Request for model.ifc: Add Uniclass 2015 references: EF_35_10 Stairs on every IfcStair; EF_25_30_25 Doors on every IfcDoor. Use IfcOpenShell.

First a look at what the model holds.

```python
import ifcopenshell

model = ifcopenshell.open("model.ifc")
print(model.schema)
print("classifications:", [c.Name for c in model.by_type("IfcClassification")])
for ifc_class in ("IfcDoor", "IfcRoof", "IfcStair", "IfcWall", "IfcWindow"):
    print(ifc_class, len(model.by_type(ifc_class)))
```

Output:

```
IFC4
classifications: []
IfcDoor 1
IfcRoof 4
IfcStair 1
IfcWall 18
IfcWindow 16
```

```python
import ifcopenshell
import ifcopenshell.api.classification

model = ifcopenshell.open("model.ifc")

system = ifcopenshell.api.classification.add_classification(model, classification="Uniclass 2015")

codes = {
    "IfcStair": ("EF_35_10", "Stairs"),
    "IfcDoor": ("EF_25_30_25", "Doors"),
}
for ifc_class, (code, name) in codes.items():
    products = model.by_type(ifc_class)
    ifcopenshell.api.classification.add_reference(
        model, products=products, classification=system, identification=code, name=name
    )
    print(code, len(products))

model.write("model_edited.ifc")
```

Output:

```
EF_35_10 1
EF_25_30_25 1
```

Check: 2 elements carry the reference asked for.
